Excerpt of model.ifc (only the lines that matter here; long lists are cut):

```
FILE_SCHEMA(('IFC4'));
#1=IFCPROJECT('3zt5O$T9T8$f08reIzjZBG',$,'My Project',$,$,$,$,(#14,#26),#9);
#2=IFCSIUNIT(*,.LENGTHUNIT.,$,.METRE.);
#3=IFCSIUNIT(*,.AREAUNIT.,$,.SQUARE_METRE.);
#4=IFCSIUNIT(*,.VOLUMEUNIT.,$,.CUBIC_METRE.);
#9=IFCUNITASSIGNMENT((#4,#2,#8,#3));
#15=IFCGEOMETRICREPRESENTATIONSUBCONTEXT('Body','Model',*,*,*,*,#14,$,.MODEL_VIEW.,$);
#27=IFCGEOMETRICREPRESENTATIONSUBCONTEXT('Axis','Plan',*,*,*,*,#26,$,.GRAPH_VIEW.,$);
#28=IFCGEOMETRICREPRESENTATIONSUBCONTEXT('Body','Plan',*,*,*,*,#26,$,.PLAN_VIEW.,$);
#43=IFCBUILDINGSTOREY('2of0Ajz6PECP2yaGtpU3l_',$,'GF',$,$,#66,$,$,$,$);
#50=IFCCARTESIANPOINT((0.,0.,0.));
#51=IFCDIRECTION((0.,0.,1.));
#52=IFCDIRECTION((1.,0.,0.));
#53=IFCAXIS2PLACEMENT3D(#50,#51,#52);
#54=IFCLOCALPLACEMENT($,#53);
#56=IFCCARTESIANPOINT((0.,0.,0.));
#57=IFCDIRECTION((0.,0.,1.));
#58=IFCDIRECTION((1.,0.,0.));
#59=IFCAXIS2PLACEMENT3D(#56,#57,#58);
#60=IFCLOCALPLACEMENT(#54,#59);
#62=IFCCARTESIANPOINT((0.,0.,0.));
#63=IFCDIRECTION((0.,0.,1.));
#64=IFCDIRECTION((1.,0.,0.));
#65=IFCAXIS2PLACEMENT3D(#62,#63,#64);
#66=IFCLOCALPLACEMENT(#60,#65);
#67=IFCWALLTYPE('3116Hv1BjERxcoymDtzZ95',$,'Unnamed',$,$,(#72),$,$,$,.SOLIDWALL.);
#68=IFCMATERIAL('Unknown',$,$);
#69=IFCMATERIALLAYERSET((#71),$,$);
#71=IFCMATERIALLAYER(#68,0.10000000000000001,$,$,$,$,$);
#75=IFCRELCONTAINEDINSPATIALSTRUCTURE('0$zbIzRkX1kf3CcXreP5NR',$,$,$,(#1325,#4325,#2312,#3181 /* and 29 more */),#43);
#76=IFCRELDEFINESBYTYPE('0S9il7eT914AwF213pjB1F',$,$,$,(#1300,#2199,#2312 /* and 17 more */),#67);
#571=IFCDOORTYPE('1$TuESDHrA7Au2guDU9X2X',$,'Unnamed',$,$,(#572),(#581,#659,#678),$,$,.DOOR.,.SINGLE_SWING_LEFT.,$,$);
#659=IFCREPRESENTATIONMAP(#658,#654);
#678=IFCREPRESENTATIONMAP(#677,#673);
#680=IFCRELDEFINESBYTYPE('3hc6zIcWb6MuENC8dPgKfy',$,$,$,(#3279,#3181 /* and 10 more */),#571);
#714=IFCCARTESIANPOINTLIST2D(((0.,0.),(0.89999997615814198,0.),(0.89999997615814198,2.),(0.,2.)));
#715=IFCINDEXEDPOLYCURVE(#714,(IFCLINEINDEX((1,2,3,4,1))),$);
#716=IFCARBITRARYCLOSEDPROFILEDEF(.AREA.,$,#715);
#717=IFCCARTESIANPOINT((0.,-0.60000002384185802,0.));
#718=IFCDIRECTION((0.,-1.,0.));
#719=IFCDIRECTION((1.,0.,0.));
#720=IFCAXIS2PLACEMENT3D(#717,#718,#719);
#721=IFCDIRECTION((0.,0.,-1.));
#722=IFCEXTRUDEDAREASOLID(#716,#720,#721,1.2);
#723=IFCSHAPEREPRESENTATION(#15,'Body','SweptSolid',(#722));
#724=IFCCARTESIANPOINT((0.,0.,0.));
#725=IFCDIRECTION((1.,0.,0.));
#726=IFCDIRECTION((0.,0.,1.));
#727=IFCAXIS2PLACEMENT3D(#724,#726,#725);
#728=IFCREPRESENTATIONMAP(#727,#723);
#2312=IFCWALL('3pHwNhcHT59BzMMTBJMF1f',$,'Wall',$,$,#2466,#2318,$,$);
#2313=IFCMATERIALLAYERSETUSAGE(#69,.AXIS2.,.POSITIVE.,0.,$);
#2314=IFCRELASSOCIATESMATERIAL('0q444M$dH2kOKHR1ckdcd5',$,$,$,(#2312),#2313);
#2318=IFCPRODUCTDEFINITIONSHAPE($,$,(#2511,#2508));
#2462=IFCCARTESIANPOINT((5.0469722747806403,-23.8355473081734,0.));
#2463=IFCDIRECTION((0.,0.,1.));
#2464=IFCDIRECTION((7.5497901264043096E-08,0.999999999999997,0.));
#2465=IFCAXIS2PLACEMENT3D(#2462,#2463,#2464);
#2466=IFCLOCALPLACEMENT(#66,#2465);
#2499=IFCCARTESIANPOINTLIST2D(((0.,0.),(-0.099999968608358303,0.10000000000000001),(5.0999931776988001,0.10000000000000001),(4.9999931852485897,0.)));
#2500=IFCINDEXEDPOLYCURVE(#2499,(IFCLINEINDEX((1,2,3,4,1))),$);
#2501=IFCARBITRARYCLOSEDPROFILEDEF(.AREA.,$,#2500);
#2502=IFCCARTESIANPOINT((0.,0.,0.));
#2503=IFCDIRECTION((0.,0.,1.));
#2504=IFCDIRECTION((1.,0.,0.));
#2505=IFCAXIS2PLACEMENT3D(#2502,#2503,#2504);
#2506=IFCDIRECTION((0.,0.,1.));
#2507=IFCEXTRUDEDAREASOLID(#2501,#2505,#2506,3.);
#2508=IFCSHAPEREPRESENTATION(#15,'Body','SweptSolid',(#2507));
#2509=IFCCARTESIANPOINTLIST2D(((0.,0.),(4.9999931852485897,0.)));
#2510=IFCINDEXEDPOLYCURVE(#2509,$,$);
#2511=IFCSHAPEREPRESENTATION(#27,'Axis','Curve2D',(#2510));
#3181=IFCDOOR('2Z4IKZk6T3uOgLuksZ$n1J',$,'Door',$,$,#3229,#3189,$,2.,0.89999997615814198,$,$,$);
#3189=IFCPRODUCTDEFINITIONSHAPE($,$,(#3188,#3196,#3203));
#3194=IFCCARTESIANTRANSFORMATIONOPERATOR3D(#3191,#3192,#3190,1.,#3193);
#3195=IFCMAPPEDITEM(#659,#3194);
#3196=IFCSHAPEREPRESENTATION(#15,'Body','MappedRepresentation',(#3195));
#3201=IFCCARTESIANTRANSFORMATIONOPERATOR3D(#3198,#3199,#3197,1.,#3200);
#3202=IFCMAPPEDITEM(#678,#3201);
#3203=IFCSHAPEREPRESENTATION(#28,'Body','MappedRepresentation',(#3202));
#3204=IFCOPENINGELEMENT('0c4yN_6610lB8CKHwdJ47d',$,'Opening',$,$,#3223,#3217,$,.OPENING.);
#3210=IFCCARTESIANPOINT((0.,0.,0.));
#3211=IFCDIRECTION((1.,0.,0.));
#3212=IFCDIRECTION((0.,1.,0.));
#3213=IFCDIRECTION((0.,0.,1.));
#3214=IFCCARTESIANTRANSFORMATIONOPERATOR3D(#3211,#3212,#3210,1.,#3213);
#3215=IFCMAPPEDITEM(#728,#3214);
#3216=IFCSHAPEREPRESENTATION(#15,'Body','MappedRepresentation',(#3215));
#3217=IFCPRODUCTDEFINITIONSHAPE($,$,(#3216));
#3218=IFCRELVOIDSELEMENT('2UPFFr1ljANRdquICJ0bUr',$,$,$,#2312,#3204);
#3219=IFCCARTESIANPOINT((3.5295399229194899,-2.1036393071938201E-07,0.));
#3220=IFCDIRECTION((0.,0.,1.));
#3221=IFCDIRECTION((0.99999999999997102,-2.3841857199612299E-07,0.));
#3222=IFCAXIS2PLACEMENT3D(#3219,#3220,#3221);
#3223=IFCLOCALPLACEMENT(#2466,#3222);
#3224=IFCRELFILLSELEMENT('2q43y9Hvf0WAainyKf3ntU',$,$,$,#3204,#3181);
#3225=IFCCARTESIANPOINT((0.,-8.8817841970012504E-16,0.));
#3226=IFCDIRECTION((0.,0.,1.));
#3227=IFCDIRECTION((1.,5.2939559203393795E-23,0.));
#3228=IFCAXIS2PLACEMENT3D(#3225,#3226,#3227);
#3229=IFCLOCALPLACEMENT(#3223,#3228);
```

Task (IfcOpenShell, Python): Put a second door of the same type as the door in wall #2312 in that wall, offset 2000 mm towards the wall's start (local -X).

```python
import ifcopenshell
import ifcopenshell.api.feature
import ifcopenshell.api.geometry
import ifcopenshell.api.root
import ifcopenshell.geom
import ifcopenshell.util.element
import ifcopenshell.util.placement
import ifcopenshell.util.shape

model = ifcopenshell.open("model.ifc")
settings = ifcopenshell.geom.settings()


def volume(element):
    """Net volume in cubic metres, openings subtracted."""
    shape = ifcopenshell.geom.create_shape(settings, element)
    return ifcopenshell.util.shape.get_volume(shape.geometry)


door = model.by_guid("2Z4IKZk6T3uOgLuksZ$n1J")
opening = door.FillsVoids[0].RelatingOpeningElement
wall = opening.VoidsElements[0].RelatingBuildingElement
before = volume(wall)
shift = ifcopenshell.util.placement.get_local_placement(wall.ObjectPlacement)[:3, 0] * -2.0

# copy_class copies the void relationship, type, container and properties, but no geometry.
new_opening = ifcopenshell.api.root.copy_class(model, product=opening)
new_opening.Representation = ifcopenshell.util.element.copy_deep(
    model, opening.Representation, exclude=["IfcGeometricRepresentationContext", "IfcRepresentationMap"]
)
new_door = ifcopenshell.api.root.copy_class(model, product=door)
new_door.Representation = ifcopenshell.util.element.copy_deep(
    model, door.Representation, exclude=["IfcGeometricRepresentationContext", "IfcRepresentationMap"]
)
ifcopenshell.api.feature.add_filling(model, opening=new_opening, element=new_door)

for old, new in ((opening, new_opening), (door, new_door)):
    matrix = ifcopenshell.util.placement.get_local_placement(old.ObjectPlacement)
    matrix[:3, 3] += shift
    ifcopenshell.api.geometry.edit_object_placement(model, product=new, matrix=matrix, is_si=False)

after = volume(wall)

print(f"wall volume {before:.3f} -> {after:.3f} m3")

model.write("model_updated.ifc")
```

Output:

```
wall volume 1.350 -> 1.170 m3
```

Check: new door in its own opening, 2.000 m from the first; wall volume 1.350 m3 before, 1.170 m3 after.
